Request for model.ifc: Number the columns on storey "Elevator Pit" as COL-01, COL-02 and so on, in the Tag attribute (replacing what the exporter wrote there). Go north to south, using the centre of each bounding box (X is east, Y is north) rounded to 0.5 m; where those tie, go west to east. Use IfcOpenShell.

First a look at what the model holds.

```python
import ifcopenshell
import ifcopenshell.util.element
import ifcopenshell.util.placement

model = ifcopenshell.open("model.ifc")
print(model.schema)
storey = next(s for s in model.by_type("IfcBuildingStorey") if s.Name == "Elevator Pit")
columns = [e for e in ifcopenshell.util.element.get_decomposition(storey) if e.is_a("IfcColumn")]
for e in sorted(columns, key=lambda e: e.id()):
    origin = ifcopenshell.util.placement.get_local_placement(e.ObjectPlacement)[:3, 3]
    print(e.id(), e.Tag, e.Name, origin.round(2) + 0.0, sep=" | ")
```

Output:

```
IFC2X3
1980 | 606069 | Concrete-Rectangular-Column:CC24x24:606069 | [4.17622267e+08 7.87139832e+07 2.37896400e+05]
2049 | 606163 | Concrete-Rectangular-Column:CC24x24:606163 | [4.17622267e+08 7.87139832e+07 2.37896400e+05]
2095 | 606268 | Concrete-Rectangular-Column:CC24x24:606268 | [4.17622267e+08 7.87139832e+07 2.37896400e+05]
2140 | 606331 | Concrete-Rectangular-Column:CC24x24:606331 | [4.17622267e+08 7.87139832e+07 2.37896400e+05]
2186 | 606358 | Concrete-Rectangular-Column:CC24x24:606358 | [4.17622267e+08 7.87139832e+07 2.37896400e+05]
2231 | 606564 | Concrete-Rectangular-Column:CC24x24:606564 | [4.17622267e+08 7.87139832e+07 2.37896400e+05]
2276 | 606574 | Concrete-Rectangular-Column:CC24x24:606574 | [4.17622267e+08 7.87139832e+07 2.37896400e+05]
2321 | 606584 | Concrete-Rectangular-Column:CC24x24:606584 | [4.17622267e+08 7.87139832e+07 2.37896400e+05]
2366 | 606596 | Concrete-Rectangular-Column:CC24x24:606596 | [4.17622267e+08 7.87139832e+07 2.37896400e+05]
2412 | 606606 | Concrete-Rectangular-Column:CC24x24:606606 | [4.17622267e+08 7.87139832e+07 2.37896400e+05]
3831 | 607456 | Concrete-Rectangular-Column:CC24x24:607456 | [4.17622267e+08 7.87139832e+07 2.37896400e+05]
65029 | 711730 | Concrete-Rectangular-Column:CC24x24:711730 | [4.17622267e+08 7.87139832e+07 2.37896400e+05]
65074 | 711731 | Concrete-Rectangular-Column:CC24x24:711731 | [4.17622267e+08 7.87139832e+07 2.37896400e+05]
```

```python
import ifcopenshell
import ifcopenshell.geom
import ifcopenshell.util.element
import ifcopenshell.util.shape

model = ifcopenshell.open("model.ifc")
settings = ifcopenshell.geom.settings()
settings.set("use-world-coords", True)


def centre(element):
    shape = ifcopenshell.geom.create_shape(settings, element)
    return ifcopenshell.util.shape.get_bbox_centroid(shape.geometry)


storey = next(s for s in model.by_type("IfcBuildingStorey") if s.Name == "Elevator Pit")
columns = [e for e in ifcopenshell.util.element.get_decomposition(storey) if e.is_a("IfcColumn")]

# Insertion points can sit at a corner or the storey origin, so sort by the geometry (in metres).
centres = {e: centre(e) for e in columns}
columns.sort(key=lambda e: (-round(centres[e][1] / 0.5), centres[e][0]))

for i, e in enumerate(columns, start=1):
    number = f"COL-{i:02d}"
    e.Tag = number
    print(e.id(), number)

model.write("model_rev.ifc")
```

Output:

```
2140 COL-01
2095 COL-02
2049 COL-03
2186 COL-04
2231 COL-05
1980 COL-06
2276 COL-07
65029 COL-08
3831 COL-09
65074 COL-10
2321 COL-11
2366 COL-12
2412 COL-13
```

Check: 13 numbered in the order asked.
